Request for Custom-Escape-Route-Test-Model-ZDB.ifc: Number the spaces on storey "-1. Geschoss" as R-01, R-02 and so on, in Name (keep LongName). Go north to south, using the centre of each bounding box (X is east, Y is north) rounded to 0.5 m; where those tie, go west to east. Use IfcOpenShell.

First a look at what the model holds.

```python
import ifcopenshell
import ifcopenshell.util.element
import ifcopenshell.util.placement

model = ifcopenshell.open("Custom-Escape-Route-Test-Model-ZDB.ifc")
print(model.schema)
storey = next(s for s in model.by_type("IfcBuildingStorey") if s.Name == "-1. Geschoss")
spaces = [e for e in ifcopenshell.util.element.get_decomposition(storey) if e.is_a("IfcSpace")]
for e in sorted(spaces, key=lambda e: e.id()):
    origin = ifcopenshell.util.placement.get_local_placement(e.ObjectPlacement)[:3, 3]
    print(e.id(), e.Name, e.LongName, origin.round(2) + 0.0, sep=" | ")
```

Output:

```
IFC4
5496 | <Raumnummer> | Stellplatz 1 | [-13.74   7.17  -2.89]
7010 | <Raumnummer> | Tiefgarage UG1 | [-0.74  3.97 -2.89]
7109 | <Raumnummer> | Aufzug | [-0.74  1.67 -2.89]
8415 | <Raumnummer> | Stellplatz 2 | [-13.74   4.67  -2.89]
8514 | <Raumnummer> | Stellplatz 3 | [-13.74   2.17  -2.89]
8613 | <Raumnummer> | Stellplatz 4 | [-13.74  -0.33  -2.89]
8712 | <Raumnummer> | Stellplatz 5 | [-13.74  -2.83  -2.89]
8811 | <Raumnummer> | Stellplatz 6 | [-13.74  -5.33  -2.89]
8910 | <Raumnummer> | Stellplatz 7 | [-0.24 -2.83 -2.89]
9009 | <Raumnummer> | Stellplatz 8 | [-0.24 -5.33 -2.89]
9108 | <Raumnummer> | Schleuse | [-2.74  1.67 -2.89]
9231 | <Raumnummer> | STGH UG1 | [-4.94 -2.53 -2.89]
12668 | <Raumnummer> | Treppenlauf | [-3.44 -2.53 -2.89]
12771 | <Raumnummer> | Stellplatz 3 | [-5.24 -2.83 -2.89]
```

```python
import ifcopenshell
import ifcopenshell.geom
import ifcopenshell.util.element
import ifcopenshell.util.shape

model = ifcopenshell.open("Custom-Escape-Route-Test-Model-ZDB.ifc")
settings = ifcopenshell.geom.settings()
settings.set("use-world-coords", True)


def centre(element):
    shape = ifcopenshell.geom.create_shape(settings, element)
    return ifcopenshell.util.shape.get_bbox_centroid(shape.geometry)


storey = next(s for s in model.by_type("IfcBuildingStorey") if s.Name == "-1. Geschoss")
spaces = [e for e in ifcopenshell.util.element.get_decomposition(storey) if e.is_a("IfcSpace")]

# Insertion points can sit at a corner or the storey origin, so sort by the geometry (in metres).
centres = {e: centre(e) for e in spaces}
spaces.sort(key=lambda e: (-round(centres[e][1] / 0.5), centres[e][0]))

for i, e in enumerate(spaces, start=1):
    number = f"R-{i:02d}"
    e.Name = number
    print(e.id(), number)

model.write("Custom-Escape-Route-Test-Model-ZDB_v2.ifc")
```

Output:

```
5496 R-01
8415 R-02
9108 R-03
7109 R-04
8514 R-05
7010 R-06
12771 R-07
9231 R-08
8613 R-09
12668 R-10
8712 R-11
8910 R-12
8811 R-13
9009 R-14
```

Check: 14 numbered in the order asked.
